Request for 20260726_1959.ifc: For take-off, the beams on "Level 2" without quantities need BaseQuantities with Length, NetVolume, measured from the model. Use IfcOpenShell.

First a look at what the model holds.

```python
import ifcopenshell
import ifcopenshell.util.element
import ifcopenshell.util.unit

model = ifcopenshell.open("20260726_1959.ifc")
print(model.schema)
for unit_type in ("LENGTHUNIT", "AREAUNIT", "VOLUMEUNIT"):
    print(unit_type, ifcopenshell.util.unit.calculate_unit_scale(model, unit_type))
storey = next(s for s in model.by_type("IfcBuildingStorey") if s.Name == "Level 2")
beams = [e for e in ifcopenshell.util.element.get_decomposition(storey) if e.is_a("IfcBeam")]
for e in sorted(beams, key=lambda e: e.id()):
    print(e.id(), e.is_a(), e.Name, list(ifcopenshell.util.element.get_psets(e, qtos_only=True)), sep=" | ")
```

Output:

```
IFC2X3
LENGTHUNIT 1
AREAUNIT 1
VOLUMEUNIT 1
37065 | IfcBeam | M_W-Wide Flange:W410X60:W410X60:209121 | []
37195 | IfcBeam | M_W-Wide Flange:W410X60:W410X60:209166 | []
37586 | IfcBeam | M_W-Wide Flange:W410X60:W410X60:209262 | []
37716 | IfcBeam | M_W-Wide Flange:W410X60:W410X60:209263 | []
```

```python
import ifcopenshell
import ifcopenshell.api.pset
import ifcopenshell.geom
import ifcopenshell.util.element
import ifcopenshell.util.shape
import ifcopenshell.util.unit

model = ifcopenshell.open("20260726_1959.ifc")
unit_scale = ifcopenshell.util.unit.calculate_unit_scale(model)
volume_scale = ifcopenshell.util.unit.calculate_unit_scale(model, "VOLUMEUNIT")
settings = ifcopenshell.geom.settings()

storey = next(s for s in model.by_type("IfcBuildingStorey") if s.Name == "Level 2")
beams = [e for e in ifcopenshell.util.element.get_decomposition(storey) if e.is_a("IfcBeam")]

for e in sorted(beams, key=lambda e: e.id()):
    if ifcopenshell.util.element.get_psets(e, qtos_only=True, should_inherit=False):
        continue
    # Geometry comes back in metres, in the element's own axes.
    shape = ifcopenshell.geom.create_shape(settings, e)
    values = {
        "Length": ifcopenshell.util.shape.get_max_xyz(shape.geometry) / unit_scale,
        "NetVolume": ifcopenshell.util.shape.get_volume(shape.geometry) / volume_scale,
    }
    qto = ifcopenshell.api.pset.add_qto(model, product=e, name="BaseQuantities")
    ifcopenshell.api.pset.edit_qto(model, qto=qto, properties=values)
    print(e.id(), {k: round(v, 3) for k, v in values.items()})

model.write("20260726_1959-out.ifc")
```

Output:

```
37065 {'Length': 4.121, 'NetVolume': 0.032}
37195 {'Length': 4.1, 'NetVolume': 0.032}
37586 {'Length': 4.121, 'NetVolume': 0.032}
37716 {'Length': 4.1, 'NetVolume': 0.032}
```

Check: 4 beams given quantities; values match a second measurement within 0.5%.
